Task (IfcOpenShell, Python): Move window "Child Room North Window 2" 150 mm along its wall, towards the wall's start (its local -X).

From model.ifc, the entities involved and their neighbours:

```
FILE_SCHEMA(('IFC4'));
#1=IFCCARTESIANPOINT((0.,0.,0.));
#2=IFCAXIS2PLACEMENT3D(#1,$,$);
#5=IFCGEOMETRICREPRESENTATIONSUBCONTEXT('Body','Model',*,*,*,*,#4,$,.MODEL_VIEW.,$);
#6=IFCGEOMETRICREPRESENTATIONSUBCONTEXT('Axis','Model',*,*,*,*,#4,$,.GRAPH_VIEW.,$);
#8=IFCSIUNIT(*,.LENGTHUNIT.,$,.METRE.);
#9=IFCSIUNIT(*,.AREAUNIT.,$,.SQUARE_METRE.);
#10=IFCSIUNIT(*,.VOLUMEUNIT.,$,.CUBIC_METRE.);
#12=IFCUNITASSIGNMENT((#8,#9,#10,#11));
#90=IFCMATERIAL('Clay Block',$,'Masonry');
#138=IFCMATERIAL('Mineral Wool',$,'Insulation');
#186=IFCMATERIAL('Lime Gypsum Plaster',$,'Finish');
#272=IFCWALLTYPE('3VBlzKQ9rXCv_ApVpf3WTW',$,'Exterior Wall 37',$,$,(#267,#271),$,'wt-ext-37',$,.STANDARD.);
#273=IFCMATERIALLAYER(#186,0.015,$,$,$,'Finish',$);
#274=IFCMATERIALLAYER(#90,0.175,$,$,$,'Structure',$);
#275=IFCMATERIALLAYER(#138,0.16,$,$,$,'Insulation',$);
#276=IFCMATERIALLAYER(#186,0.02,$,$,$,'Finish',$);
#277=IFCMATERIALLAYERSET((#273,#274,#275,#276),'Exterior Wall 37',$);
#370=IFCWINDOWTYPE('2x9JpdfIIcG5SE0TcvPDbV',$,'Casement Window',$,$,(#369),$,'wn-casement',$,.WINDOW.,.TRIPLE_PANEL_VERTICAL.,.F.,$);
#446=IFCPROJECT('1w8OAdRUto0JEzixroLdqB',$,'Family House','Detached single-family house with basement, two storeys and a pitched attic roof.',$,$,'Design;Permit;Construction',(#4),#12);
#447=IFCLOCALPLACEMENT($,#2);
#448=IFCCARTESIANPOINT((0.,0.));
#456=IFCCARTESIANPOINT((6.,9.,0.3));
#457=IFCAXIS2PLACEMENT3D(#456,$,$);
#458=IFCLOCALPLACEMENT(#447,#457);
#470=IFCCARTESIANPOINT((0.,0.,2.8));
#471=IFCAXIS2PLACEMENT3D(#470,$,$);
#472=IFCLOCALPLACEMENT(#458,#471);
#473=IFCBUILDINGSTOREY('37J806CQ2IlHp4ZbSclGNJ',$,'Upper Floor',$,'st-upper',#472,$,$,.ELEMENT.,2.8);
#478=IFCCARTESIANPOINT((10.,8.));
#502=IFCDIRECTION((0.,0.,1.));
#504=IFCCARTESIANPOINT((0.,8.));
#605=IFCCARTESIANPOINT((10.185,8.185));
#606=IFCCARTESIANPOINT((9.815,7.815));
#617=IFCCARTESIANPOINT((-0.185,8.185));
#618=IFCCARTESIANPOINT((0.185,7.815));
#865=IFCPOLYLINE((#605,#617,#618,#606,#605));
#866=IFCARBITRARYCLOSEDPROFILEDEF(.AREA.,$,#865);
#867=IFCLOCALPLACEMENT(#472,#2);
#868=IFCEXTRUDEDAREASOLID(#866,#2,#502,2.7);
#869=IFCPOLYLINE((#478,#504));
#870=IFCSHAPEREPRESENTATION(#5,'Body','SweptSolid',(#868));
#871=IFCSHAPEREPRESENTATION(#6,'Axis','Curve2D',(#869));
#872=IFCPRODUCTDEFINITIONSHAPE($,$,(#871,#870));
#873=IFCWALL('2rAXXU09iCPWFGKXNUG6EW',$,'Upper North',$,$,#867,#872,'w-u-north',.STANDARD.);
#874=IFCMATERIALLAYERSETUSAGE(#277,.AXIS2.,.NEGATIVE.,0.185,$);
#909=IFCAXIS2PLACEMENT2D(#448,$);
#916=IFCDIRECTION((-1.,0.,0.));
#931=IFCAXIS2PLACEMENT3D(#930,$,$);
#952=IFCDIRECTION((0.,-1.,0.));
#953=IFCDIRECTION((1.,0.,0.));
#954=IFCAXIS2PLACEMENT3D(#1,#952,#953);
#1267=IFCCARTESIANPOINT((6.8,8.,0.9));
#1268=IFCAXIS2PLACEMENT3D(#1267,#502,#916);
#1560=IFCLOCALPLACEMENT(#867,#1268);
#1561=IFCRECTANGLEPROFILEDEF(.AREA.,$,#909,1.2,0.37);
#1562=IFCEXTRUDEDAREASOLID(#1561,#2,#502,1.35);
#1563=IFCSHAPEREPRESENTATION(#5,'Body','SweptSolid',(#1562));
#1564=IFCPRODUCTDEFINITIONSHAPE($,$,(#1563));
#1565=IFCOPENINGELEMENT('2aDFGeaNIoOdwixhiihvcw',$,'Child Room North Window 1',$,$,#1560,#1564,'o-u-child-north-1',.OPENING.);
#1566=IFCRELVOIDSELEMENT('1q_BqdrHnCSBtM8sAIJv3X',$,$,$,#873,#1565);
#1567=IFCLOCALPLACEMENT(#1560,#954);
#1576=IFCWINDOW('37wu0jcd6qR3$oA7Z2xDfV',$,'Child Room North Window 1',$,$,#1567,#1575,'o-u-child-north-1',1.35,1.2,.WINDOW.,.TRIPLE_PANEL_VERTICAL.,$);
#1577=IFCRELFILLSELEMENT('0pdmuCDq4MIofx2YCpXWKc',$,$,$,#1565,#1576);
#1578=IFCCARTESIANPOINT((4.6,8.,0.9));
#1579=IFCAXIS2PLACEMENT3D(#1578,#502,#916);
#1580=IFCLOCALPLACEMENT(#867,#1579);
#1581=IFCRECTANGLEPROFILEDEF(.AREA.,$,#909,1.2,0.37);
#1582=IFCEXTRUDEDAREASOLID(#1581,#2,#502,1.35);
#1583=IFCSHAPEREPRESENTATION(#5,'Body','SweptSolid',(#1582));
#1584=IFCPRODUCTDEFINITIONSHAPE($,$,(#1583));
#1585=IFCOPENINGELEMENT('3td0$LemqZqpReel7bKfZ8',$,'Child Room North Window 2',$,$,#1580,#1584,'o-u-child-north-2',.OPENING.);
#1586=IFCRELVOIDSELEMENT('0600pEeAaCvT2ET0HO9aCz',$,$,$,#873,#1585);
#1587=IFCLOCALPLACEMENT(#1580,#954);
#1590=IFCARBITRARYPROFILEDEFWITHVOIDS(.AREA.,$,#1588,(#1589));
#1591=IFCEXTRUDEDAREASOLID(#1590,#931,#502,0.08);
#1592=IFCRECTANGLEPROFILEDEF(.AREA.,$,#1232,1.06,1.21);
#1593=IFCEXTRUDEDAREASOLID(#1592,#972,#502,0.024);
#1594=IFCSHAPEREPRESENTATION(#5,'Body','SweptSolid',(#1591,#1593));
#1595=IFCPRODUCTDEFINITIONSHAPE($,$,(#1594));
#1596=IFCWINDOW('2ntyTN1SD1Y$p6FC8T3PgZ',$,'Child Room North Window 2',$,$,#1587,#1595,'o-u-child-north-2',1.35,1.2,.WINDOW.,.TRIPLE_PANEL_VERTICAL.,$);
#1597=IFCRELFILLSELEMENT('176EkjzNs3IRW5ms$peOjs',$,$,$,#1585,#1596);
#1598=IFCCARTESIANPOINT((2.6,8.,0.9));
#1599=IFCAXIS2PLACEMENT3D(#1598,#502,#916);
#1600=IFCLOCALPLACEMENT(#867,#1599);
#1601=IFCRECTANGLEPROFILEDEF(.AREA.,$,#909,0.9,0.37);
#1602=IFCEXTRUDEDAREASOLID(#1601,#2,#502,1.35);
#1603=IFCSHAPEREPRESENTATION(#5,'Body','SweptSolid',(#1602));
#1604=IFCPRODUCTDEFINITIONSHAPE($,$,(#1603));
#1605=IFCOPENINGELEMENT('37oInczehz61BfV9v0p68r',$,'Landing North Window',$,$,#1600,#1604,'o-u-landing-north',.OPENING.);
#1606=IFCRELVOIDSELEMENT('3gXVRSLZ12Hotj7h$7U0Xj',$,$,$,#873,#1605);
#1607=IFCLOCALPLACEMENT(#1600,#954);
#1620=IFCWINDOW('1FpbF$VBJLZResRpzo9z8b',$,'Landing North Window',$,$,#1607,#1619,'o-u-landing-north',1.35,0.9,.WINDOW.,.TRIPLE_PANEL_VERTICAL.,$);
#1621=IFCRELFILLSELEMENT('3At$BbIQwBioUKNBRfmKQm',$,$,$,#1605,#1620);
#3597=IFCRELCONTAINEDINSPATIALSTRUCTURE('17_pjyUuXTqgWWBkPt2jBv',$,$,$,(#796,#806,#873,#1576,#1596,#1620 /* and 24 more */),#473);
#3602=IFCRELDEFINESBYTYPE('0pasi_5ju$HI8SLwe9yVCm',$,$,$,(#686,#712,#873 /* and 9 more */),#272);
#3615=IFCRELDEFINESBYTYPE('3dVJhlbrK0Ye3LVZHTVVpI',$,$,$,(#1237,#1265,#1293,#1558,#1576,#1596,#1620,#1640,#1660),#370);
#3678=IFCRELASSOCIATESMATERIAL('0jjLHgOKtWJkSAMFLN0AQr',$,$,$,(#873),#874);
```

```python
import ifcopenshell
import ifcopenshell.api.geometry
import ifcopenshell.util.placement
import ifcopenshell.util.unit

model = ifcopenshell.open("model.ifc")
unit_scale = ifcopenshell.util.unit.calculate_unit_scale(model)

window = model.by_id(1596)
opening = window.FillsVoids[0].RelatingOpeningElement
wall = opening.VoidsElements[0].RelatingBuildingElement

wall_matrix = ifcopenshell.util.placement.get_local_placement(wall.ObjectPlacement)
shift = wall_matrix[:3, 0] * -0.15 / unit_scale
before = ifcopenshell.util.placement.get_local_placement(window.ObjectPlacement)[:3, 3].copy()

# The window is placed relative to its opening, so it follows when the opening moves.
matrix = ifcopenshell.util.placement.get_local_placement(opening.ObjectPlacement)
matrix[:3, 3] += shift
ifcopenshell.api.geometry.edit_object_placement(
    model, product=opening, matrix=matrix, is_si=False, should_transform_children=True
)

after = ifcopenshell.util.placement.get_local_placement(window.ObjectPlacement)[:3, 3]
print("window moved by", (after - before).round(3) + 0.0)

model.write("model-out.ifc")
```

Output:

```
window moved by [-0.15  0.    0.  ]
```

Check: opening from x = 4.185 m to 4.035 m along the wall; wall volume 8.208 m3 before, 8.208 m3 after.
